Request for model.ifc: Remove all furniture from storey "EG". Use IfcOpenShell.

First a look at what the model holds.

```python
import ifcopenshell
import ifcopenshell.util.element

model = ifcopenshell.open("model.ifc")
print(model.schema)
storey = next(s for s in model.by_type("IfcBuildingStorey") if s.Name == "EG")
furniture = [e for e in ifcopenshell.util.element.get_decomposition(storey) if e.is_a("IfcFurnishingElement")]
seen = {}
for e in furniture:
    element_type = ifcopenshell.util.element.get_type(e)
    name = element_type.Name if element_type not in (None, e) else None
    seen[name] = seen.get(name, 0) + 1
for name, count in sorted(seen.items(), key=str):
    print(count, "x", name)
```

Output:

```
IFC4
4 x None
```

```python
import ifcopenshell
import ifcopenshell.api.root
import ifcopenshell.util.element

model = ifcopenshell.open("model.ifc")

storey = next(s for s in model.by_type("IfcBuildingStorey") if s.Name == "EG")
furniture = [e for e in ifcopenshell.util.element.get_decomposition(storey) if e.is_a("IfcFurnishingElement")]

for e in furniture:
    ifcopenshell.api.root.remove_product(model, product=e)
print(len(furniture), "removed")

model.write("model_v2.ifc")
```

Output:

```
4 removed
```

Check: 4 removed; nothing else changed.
